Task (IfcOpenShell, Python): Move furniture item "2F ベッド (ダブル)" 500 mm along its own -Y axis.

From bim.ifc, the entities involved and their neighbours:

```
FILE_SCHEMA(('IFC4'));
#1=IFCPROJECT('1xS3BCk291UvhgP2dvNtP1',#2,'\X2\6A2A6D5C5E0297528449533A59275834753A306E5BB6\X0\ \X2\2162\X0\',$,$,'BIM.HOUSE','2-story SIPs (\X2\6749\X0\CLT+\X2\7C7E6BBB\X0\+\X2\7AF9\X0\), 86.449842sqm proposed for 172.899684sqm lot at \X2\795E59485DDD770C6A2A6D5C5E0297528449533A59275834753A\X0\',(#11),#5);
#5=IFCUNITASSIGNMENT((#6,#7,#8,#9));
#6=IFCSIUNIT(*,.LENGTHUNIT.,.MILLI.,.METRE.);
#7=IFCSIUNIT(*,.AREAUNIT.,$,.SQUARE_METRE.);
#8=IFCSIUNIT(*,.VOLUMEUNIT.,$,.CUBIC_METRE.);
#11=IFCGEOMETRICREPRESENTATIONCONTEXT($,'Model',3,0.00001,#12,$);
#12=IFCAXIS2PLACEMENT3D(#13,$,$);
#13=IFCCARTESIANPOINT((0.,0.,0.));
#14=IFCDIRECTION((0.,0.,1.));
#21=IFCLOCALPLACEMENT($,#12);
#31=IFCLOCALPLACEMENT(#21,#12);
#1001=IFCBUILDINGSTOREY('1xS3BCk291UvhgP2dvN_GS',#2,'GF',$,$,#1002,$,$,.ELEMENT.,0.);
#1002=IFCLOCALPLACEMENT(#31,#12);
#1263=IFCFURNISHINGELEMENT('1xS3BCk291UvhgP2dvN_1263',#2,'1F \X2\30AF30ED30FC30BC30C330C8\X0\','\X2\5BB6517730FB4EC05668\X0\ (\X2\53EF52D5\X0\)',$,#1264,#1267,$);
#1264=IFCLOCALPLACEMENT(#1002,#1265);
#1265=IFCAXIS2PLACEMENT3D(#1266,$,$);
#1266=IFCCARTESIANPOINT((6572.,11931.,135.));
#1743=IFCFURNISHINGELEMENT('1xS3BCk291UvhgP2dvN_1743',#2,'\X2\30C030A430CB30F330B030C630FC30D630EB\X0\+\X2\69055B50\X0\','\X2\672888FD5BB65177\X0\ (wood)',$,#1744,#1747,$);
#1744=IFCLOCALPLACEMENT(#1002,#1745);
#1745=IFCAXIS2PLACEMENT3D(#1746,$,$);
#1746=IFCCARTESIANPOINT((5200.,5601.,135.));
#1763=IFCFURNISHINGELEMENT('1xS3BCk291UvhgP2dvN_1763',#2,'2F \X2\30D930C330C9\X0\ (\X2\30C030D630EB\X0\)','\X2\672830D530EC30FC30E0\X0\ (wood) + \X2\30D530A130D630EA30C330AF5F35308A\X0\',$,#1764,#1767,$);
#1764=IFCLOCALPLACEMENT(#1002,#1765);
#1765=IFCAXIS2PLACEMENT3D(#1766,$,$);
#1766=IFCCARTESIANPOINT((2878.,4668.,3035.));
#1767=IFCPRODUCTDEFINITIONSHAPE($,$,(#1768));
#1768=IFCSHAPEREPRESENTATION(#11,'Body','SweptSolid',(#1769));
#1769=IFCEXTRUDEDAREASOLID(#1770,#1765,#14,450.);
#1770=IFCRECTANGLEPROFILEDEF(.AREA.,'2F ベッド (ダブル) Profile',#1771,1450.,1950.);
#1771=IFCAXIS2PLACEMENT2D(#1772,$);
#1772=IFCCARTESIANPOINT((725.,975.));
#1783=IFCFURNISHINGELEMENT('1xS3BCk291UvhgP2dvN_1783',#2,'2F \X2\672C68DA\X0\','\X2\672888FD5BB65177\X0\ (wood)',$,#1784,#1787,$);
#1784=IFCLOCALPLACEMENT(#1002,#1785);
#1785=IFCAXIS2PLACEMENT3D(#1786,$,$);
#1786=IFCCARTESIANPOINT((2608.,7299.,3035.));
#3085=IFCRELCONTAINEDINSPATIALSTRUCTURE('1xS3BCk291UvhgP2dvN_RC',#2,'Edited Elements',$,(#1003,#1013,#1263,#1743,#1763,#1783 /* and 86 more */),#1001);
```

```python
import ifcopenshell
import ifcopenshell.api.geometry
import ifcopenshell.util.placement
import ifcopenshell.util.unit

model = ifcopenshell.open("bim.ifc")
unit_scale = ifcopenshell.util.unit.calculate_unit_scale(model)

item = model.by_guid("1xS3BCk291UvhgP2dvN_1763")
matrix = ifcopenshell.util.placement.get_local_placement(item.ObjectPlacement)
matrix[:3, 3] -= matrix[:3, 1] * 0.5 / unit_scale
ifcopenshell.api.geometry.edit_object_placement(model, product=item, matrix=matrix, is_si=False)

print(ifcopenshell.util.placement.get_local_placement(item.ObjectPlacement).round(3) + 0.0)

model.write("bim-out.ifc")
```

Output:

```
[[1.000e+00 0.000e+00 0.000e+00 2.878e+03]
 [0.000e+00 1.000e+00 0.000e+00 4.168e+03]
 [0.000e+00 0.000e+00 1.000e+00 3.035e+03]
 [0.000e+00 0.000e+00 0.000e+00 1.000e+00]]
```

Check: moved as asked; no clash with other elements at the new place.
